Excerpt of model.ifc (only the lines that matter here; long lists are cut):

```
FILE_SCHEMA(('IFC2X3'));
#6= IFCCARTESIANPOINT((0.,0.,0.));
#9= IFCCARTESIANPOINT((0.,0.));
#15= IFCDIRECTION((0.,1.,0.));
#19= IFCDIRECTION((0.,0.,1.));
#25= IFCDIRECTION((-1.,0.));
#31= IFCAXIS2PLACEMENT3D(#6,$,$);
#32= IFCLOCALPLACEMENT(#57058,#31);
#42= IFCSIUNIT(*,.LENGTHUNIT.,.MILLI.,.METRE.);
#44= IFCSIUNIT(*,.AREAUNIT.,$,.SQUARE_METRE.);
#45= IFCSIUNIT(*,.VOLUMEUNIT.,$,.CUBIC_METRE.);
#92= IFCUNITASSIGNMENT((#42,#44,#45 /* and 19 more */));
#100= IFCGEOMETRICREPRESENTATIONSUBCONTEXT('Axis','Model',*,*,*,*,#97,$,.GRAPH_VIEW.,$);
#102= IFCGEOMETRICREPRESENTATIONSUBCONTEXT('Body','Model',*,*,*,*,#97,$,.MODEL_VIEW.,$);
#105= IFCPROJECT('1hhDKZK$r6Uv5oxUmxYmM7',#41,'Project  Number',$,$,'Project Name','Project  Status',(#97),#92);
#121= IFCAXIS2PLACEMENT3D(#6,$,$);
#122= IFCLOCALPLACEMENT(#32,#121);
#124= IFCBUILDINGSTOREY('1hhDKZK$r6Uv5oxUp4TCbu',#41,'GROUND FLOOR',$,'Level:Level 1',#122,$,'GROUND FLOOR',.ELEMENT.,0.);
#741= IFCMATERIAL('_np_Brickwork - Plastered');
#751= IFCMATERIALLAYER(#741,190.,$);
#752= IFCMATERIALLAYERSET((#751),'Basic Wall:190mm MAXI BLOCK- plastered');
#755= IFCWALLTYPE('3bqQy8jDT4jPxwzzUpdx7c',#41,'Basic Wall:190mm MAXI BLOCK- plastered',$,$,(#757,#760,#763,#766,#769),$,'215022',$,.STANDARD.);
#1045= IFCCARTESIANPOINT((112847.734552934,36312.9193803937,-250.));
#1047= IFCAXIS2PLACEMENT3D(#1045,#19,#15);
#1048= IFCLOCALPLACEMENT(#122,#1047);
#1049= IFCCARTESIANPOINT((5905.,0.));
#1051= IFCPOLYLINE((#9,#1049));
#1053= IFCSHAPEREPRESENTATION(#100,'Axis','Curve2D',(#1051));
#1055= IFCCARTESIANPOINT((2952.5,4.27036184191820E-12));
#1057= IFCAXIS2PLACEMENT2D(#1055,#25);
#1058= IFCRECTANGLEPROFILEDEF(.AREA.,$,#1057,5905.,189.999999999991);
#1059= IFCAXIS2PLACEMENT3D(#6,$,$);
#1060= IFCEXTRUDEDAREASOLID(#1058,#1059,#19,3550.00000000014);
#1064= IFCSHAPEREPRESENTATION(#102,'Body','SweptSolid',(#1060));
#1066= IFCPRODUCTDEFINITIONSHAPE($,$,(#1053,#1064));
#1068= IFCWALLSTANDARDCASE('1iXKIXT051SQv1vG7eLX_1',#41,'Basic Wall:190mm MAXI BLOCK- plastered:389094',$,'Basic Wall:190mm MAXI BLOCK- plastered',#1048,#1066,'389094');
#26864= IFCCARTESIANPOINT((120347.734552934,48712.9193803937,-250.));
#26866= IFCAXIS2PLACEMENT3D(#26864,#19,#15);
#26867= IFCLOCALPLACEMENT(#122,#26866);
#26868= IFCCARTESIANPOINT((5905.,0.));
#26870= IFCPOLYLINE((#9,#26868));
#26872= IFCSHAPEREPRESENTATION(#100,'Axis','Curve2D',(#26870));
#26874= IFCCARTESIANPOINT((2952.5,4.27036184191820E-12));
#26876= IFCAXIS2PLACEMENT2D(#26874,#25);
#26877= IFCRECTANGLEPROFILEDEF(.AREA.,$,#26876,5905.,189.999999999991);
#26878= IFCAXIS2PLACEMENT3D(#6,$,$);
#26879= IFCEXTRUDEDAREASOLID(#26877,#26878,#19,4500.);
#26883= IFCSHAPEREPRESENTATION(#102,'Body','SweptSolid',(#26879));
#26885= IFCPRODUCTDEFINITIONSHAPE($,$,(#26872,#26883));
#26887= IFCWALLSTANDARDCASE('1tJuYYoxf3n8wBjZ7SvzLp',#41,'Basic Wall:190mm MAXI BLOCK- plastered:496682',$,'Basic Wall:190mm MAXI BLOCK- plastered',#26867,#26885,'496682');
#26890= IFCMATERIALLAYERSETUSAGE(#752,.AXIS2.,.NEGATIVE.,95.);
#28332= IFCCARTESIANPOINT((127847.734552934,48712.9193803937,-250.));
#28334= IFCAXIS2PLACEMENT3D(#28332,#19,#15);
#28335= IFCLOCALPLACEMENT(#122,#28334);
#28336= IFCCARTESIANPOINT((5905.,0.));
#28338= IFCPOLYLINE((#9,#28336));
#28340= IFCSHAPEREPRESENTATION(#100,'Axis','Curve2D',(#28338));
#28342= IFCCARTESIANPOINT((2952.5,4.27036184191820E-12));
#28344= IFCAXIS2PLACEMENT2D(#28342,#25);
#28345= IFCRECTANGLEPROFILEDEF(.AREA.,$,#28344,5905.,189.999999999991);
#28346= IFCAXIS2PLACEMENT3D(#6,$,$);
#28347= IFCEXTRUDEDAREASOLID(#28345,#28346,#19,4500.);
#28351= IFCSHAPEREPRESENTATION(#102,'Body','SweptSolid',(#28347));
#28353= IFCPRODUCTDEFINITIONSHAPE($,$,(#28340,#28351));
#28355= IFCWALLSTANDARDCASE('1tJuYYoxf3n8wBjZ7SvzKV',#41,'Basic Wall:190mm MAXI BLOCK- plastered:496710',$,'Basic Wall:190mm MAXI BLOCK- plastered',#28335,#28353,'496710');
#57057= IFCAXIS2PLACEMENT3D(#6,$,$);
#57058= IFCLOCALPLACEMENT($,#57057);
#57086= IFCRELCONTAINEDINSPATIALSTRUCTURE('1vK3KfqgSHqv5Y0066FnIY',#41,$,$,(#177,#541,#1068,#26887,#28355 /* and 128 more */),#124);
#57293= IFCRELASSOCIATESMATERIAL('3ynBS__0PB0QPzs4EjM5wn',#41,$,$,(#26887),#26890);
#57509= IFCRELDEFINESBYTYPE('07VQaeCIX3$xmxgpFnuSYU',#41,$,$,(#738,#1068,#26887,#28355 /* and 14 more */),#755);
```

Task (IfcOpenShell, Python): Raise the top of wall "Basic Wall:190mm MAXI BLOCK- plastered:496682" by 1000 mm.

```python
import ifcopenshell
import ifcopenshell.geom
import ifcopenshell.util.representation
import ifcopenshell.util.shape

model = ifcopenshell.open("model.ifc")
settings = ifcopenshell.geom.settings()


def volume(element):
    """Net volume in cubic metres, openings subtracted."""
    shape = ifcopenshell.geom.create_shape(settings, element)
    return ifcopenshell.util.shape.get_volume(shape.geometry)


wall = model.by_guid("1tJuYYoxf3n8wBjZ7SvzLp")
before = volume(wall)

body = ifcopenshell.util.representation.get_representation(wall, "Model", "Body")
solid = body.Items[0]
old_height = solid.Depth
solid.Depth += 1000.0
after = volume(wall)

print(f"height {old_height:g} -> {solid.Depth:g}, volume {before:.3f} -> {after:.3f} m3")

model.write("model_edited.ifc")
```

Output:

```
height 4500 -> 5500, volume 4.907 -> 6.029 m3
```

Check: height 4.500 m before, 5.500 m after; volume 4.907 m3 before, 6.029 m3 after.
